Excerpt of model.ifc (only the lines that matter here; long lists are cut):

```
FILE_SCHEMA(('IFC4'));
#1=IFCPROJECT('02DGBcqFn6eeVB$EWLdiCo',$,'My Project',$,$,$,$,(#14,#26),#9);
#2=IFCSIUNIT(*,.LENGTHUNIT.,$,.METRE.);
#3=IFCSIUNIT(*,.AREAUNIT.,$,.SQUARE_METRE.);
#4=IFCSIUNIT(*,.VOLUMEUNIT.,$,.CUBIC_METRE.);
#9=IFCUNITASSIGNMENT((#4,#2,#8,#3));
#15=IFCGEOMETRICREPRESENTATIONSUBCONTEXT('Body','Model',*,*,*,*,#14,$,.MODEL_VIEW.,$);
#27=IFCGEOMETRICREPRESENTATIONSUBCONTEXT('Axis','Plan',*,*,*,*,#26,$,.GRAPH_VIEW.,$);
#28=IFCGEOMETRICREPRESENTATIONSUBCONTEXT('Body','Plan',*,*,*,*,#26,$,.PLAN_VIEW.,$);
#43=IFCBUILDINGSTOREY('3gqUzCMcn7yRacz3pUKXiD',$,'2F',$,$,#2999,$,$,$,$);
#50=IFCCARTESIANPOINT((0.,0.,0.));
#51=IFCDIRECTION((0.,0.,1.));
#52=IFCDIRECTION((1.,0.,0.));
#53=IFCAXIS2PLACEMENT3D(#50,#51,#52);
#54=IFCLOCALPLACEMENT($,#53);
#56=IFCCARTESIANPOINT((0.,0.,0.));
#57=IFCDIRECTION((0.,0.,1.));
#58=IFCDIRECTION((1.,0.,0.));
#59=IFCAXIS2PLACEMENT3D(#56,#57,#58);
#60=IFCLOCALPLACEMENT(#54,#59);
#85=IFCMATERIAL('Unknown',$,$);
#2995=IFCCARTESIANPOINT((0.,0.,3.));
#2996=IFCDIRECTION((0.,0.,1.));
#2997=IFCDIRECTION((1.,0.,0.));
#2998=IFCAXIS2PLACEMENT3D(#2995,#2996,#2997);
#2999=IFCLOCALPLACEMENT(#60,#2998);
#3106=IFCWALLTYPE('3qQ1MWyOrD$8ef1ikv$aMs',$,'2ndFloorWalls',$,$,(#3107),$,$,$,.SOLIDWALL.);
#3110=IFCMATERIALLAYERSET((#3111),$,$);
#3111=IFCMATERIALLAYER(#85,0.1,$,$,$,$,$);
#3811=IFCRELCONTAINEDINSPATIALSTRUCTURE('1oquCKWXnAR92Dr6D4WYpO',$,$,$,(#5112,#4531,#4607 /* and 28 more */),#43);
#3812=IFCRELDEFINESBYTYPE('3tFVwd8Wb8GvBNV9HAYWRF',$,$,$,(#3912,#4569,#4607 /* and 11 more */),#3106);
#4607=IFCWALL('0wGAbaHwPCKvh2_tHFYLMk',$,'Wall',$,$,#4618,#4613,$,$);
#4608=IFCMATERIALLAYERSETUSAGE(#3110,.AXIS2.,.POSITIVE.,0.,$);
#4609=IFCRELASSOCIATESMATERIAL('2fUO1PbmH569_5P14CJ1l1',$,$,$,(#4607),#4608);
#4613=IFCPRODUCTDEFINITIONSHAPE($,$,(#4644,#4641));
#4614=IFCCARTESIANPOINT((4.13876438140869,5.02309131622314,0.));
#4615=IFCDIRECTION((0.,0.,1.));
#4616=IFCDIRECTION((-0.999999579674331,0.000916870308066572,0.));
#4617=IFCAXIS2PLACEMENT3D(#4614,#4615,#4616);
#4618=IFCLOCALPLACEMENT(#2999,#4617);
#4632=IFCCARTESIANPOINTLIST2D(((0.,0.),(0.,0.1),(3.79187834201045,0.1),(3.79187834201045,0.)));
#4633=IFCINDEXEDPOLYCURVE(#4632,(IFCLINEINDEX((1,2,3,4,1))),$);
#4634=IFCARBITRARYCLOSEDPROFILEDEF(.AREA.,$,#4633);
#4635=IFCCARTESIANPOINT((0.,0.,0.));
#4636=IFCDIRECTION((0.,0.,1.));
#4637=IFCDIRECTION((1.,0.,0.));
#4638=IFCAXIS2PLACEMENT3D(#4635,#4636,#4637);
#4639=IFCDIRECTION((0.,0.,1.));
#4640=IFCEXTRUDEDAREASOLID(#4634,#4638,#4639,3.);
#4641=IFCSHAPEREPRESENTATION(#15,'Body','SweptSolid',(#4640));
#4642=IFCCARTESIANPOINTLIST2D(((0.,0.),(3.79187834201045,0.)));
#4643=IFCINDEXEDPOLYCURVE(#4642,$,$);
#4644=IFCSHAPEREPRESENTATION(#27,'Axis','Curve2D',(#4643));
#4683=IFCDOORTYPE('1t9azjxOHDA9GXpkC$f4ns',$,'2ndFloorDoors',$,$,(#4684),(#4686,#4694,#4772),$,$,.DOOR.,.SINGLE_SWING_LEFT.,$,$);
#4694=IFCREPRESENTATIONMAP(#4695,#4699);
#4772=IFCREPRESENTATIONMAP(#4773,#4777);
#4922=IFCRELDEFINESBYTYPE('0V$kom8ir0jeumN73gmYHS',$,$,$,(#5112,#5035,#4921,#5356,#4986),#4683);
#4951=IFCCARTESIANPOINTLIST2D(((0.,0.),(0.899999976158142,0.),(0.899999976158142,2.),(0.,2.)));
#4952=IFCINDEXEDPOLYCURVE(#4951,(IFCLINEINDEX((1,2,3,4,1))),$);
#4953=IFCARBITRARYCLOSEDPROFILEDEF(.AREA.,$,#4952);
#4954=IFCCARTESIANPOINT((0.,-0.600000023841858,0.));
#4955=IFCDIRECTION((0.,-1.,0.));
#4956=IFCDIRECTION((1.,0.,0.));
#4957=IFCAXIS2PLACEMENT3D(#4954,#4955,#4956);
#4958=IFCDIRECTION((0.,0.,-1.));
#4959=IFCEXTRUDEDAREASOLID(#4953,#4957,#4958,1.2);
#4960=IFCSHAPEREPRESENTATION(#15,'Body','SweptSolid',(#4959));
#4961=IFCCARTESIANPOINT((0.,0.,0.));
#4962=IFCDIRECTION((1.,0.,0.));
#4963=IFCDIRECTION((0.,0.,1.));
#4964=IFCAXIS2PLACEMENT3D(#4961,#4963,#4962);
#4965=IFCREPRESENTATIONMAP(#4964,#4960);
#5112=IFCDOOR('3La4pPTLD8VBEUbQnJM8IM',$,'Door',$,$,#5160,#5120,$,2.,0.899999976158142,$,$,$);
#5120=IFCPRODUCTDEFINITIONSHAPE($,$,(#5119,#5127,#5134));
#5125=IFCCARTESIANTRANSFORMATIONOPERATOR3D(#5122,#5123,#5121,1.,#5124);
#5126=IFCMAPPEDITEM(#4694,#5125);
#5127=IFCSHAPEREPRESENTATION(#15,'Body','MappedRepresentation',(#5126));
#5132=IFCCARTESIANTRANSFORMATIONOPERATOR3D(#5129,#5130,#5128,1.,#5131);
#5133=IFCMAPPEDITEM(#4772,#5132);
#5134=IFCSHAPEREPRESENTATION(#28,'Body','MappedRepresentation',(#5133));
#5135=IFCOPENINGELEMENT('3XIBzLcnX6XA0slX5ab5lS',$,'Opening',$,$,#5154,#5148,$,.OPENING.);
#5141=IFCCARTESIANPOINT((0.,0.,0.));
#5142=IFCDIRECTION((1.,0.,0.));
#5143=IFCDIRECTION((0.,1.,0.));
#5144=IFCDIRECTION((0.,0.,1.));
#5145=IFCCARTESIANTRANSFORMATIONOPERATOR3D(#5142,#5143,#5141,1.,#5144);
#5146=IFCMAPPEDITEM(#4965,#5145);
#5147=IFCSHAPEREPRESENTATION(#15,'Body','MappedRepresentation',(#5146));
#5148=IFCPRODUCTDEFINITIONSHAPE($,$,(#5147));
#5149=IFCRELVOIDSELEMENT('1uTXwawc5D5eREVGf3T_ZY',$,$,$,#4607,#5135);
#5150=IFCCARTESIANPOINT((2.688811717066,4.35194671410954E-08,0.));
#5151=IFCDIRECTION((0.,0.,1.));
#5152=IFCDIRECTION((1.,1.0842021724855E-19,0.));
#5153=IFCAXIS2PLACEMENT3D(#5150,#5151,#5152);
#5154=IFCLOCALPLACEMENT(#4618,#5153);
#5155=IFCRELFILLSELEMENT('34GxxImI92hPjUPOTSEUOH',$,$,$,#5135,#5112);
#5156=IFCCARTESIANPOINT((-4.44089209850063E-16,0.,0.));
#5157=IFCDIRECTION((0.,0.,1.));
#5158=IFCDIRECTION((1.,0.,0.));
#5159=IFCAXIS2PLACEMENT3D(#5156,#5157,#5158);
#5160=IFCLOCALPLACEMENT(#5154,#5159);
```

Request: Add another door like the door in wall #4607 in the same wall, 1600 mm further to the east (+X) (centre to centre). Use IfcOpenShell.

```python
import ifcopenshell
import ifcopenshell.api.feature
import ifcopenshell.api.geometry
import ifcopenshell.api.root
import ifcopenshell.geom
import ifcopenshell.util.element
import ifcopenshell.util.placement
import ifcopenshell.util.shape
import ifcopenshell.util.unit

model = ifcopenshell.open("model.ifc")
unit_scale = ifcopenshell.util.unit.calculate_unit_scale(model)
settings = ifcopenshell.geom.settings()


def volume(element):
    """Net volume in cubic metres, openings subtracted."""
    shape = ifcopenshell.geom.create_shape(settings, element)
    return ifcopenshell.util.shape.get_volume(shape.geometry)


door = model.by_guid("3La4pPTLD8VBEUbQnJM8IM")
opening = door.FillsVoids[0].RelatingOpeningElement
wall = opening.VoidsElements[0].RelatingBuildingElement
before = volume(wall)
shift = ifcopenshell.util.placement.get_local_placement(wall.ObjectPlacement)[:3, 0] * -1.6 / unit_scale

# copy_class copies the void relationship, type, container and properties, but no geometry.
new_opening = ifcopenshell.api.root.copy_class(model, product=opening)
new_opening.Representation = ifcopenshell.util.element.copy_deep(
    model, opening.Representation, exclude=["IfcGeometricRepresentationContext", "IfcRepresentationMap"]
)
new_door = ifcopenshell.api.root.copy_class(model, product=door)
new_door.Representation = ifcopenshell.util.element.copy_deep(
    model, door.Representation, exclude=["IfcGeometricRepresentationContext", "IfcRepresentationMap"]
)
ifcopenshell.api.feature.add_filling(model, opening=new_opening, element=new_door)

for old, new in ((opening, new_opening), (door, new_door)):
    matrix = ifcopenshell.util.placement.get_local_placement(old.ObjectPlacement)
    matrix[:3, 3] += shift
    ifcopenshell.api.geometry.edit_object_placement(model, product=new, matrix=matrix, is_si=False)

after = volume(wall)

print(f"wall volume {before:.3f} -> {after:.3f} m3")

model.write("model-out.ifc")
```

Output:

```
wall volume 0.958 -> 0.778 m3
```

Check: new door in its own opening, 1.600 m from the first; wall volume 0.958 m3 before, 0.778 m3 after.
